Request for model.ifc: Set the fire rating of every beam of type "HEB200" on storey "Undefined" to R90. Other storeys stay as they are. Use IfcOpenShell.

First a look at what the model holds.

```python
import ifcopenshell
import ifcopenshell.util.element

model = ifcopenshell.open("model.ifc")
print(model.schema)
storey = next(s for s in model.by_type("IfcBuildingStorey") if s.Name == "Undefined")
beams = [e for e in ifcopenshell.util.element.get_decomposition(storey) if e.is_a("IfcBeam")]
seen = {}
for e in beams:
    element_type = ifcopenshell.util.element.get_type(e)
    key = (element_type.Name if element_type != e and element_type else None, ifcopenshell.util.element.get_pset(e, "Pset_BeamCommon", "FireRating"))
    seen[key] = seen.get(key, 0) + 1
for (name, value), count in sorted(seen.items(), key=str):
    print(count, "x", name, "|", value)
```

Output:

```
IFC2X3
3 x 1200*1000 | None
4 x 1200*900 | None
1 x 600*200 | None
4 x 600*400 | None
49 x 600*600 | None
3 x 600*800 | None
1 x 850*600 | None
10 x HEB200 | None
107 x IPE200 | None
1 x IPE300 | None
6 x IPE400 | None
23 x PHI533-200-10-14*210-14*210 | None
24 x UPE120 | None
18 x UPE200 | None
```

```python
import ifcopenshell
import ifcopenshell.api.pset
import ifcopenshell.util.element

model = ifcopenshell.open("model.ifc")

storey = next(s for s in model.by_type("IfcBuildingStorey") if s.Name == "Undefined")
beams = [e for e in ifcopenshell.util.element.get_decomposition(storey) if e.is_a("IfcBeam")]

count = 0
for e in beams:
    element_type = ifcopenshell.util.element.get_type(e)
    if element_type in (None, e) or element_type.Name != "HEB200":
        continue
    # add_pset returns the element's existing set when there is one.
    pset = ifcopenshell.api.pset.add_pset(model, product=e, name="Pset_BeamCommon")
    ifcopenshell.api.pset.edit_pset(model, pset=pset, properties={"FireRating": "R90"})
    count += 1

print(count, "beams updated")

model.write("model_updated.ifc")
```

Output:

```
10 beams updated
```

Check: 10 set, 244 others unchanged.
